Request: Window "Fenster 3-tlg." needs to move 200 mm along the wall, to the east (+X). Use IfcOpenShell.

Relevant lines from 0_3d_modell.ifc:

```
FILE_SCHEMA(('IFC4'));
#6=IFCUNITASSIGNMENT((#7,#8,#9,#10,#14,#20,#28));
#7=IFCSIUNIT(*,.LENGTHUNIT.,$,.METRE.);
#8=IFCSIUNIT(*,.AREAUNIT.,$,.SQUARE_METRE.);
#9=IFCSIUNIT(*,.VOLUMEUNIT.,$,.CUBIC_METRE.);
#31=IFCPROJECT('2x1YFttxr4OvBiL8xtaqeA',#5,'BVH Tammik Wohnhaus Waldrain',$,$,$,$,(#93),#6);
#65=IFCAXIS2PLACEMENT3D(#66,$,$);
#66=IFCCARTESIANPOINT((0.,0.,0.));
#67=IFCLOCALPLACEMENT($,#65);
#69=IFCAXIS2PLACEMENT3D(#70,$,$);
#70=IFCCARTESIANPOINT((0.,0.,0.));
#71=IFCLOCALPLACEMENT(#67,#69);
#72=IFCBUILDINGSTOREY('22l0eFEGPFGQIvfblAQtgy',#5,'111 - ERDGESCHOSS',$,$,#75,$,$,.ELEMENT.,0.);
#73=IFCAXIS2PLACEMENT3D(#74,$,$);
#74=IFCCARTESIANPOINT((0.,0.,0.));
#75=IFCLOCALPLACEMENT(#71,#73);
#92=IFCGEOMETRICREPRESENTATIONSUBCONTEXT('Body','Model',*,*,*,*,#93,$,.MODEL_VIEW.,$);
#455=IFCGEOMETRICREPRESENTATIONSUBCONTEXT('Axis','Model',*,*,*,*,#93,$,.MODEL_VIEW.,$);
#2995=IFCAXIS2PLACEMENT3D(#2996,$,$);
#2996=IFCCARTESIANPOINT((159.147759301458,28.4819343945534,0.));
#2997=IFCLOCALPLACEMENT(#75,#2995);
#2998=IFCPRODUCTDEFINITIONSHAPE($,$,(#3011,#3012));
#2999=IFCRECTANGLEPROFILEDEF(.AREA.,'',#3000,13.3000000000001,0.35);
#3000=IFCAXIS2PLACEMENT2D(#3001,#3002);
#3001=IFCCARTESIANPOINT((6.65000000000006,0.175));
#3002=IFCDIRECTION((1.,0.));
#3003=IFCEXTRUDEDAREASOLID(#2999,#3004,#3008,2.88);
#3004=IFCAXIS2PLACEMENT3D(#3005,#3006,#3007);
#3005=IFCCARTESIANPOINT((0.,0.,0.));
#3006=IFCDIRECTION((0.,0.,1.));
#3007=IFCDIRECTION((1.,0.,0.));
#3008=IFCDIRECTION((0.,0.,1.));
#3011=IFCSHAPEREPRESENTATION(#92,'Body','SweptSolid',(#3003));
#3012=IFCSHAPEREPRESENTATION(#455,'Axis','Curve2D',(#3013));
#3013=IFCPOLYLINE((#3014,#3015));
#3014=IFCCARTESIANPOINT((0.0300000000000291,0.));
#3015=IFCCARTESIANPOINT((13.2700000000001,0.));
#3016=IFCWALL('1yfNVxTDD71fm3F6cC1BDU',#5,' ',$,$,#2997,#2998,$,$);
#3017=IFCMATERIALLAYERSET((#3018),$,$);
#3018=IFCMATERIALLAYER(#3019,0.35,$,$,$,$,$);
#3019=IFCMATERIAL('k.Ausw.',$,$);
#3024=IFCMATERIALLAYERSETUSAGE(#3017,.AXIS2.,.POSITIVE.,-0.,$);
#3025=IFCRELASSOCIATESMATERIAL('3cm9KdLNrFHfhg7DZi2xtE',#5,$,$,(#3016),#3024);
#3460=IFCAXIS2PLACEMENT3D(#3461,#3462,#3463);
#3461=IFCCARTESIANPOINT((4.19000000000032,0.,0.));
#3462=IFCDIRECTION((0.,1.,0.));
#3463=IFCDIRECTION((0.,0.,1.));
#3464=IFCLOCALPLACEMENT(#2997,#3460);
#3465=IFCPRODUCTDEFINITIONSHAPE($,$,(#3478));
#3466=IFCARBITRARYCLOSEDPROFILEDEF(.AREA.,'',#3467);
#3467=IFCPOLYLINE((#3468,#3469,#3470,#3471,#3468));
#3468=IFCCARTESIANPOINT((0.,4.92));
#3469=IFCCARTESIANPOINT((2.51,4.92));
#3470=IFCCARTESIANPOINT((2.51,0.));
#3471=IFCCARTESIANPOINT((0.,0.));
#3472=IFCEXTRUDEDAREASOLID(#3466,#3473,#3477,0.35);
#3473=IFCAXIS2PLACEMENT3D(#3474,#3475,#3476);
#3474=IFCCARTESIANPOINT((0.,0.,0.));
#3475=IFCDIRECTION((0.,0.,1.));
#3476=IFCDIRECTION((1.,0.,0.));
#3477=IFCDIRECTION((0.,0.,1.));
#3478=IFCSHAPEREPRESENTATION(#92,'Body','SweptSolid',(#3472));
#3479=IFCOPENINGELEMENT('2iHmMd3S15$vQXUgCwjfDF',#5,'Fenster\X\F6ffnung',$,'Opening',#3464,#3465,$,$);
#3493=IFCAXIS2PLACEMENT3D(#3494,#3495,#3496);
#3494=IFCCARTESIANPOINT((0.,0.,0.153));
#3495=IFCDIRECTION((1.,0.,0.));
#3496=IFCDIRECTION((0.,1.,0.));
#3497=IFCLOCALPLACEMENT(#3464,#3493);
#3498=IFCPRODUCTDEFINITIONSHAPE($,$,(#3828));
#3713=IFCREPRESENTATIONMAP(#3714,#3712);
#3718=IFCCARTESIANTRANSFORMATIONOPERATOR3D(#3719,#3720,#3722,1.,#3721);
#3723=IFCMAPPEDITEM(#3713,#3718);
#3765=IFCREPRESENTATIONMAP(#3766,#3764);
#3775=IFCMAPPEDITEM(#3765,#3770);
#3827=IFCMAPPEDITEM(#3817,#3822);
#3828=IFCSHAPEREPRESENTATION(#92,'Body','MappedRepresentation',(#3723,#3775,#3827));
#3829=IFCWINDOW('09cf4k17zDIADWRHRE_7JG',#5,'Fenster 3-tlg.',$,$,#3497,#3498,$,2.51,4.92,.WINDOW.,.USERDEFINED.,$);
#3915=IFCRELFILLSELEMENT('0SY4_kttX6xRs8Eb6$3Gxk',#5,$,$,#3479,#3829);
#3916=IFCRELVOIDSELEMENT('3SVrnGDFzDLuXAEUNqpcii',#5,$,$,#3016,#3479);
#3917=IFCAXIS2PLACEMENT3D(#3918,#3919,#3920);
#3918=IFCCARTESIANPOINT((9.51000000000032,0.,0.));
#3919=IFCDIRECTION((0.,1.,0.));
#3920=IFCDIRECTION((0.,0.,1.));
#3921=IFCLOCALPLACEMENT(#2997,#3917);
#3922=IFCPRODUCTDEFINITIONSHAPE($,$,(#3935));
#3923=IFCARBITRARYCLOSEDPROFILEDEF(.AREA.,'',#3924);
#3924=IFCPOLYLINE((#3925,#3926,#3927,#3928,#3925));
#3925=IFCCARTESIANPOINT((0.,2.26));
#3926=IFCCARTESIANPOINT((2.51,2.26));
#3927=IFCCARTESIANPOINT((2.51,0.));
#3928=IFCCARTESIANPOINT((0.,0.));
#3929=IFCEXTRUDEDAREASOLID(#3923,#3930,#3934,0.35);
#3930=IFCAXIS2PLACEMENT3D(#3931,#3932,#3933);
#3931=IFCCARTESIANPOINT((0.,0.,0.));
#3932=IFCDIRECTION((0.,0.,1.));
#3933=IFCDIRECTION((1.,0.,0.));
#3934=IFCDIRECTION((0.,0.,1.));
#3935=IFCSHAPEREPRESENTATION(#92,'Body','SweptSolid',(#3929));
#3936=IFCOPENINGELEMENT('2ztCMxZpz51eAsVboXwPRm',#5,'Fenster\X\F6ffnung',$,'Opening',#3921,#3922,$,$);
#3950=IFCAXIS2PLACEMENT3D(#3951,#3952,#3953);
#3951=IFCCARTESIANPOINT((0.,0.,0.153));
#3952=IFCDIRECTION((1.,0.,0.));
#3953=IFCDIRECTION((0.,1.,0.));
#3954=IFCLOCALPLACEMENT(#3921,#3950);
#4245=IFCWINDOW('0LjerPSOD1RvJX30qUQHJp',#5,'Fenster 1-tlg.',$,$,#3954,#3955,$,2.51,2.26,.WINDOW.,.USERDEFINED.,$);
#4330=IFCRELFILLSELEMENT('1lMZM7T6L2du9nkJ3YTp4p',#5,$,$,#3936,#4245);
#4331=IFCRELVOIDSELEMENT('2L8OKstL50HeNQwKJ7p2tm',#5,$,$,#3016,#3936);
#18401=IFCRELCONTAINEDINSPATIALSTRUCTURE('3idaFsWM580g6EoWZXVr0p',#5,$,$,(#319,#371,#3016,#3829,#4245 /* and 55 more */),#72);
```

```python
import ifcopenshell
import ifcopenshell.api.geometry
import ifcopenshell.util.placement
import ifcopenshell.util.unit

model = ifcopenshell.open("0_3d_modell.ifc")
unit_scale = ifcopenshell.util.unit.calculate_unit_scale(model)

window = model.by_guid("09cf4k17zDIADWRHRE_7JG")
opening = window.FillsVoids[0].RelatingOpeningElement
wall = opening.VoidsElements[0].RelatingBuildingElement

wall_matrix = ifcopenshell.util.placement.get_local_placement(wall.ObjectPlacement)
shift = wall_matrix[:3, 0] * 0.2 / unit_scale
before = ifcopenshell.util.placement.get_local_placement(window.ObjectPlacement)[:3, 3].copy()

# The window is placed relative to its opening, so it follows when the opening moves.
matrix = ifcopenshell.util.placement.get_local_placement(opening.ObjectPlacement)
matrix[:3, 3] += shift
ifcopenshell.api.geometry.edit_object_placement(
    model, product=opening, matrix=matrix, is_si=False, should_transform_children=True
)

after = ifcopenshell.util.placement.get_local_placement(window.ObjectPlacement)[:3, 3]
print("window moved by", (after - before).round(3) + 0.0)

model.write("0_3d_modell_edited.ifc")
```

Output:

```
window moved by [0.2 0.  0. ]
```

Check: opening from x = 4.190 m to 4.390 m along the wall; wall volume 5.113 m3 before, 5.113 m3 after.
